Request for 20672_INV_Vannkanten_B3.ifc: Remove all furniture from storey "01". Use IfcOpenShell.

First a look at what the model holds.

```python
import ifcopenshell
import ifcopenshell.util.element

model = ifcopenshell.open("20672_INV_Vannkanten_B3.ifc")
print(model.schema)
storey = next(s for s in model.by_type("IfcBuildingStorey") if s.Name == "01")
furniture = [e for e in ifcopenshell.util.element.get_decomposition(storey) if e.is_a("IfcFurnishingElement")]
seen = {}
for e in furniture:
    element_type = ifcopenshell.util.element.get_type(e)
    name = element_type.Name if element_type not in (None, e) else None
    seen[name] = seen.get(name, 0) + 1
for name, count in sorted(seen.items(), key=str):
    print(count, "x", name)
```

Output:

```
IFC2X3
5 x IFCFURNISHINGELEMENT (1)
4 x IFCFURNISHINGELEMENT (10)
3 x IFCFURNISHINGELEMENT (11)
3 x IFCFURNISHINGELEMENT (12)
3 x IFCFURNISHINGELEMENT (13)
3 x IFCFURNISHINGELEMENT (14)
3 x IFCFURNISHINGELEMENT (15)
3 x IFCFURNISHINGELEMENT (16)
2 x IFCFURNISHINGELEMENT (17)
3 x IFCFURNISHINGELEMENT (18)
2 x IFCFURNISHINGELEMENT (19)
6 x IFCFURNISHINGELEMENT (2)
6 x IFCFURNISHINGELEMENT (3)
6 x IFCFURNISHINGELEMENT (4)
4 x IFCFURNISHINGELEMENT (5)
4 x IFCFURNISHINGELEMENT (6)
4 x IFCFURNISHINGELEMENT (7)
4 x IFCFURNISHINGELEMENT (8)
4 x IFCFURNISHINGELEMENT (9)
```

```python
import ifcopenshell
import ifcopenshell.api.root
import ifcopenshell.util.element

model = ifcopenshell.open("20672_INV_Vannkanten_B3.ifc")

storey = next(s for s in model.by_type("IfcBuildingStorey") if s.Name == "01")
furniture = [e for e in ifcopenshell.util.element.get_decomposition(storey) if e.is_a("IfcFurnishingElement")]

for e in furniture:
    ifcopenshell.api.root.remove_product(model, product=e)
print(len(furniture), "removed")

model.write("20672_INV_Vannkanten_B3_rev.ifc")
```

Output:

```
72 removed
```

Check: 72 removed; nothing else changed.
